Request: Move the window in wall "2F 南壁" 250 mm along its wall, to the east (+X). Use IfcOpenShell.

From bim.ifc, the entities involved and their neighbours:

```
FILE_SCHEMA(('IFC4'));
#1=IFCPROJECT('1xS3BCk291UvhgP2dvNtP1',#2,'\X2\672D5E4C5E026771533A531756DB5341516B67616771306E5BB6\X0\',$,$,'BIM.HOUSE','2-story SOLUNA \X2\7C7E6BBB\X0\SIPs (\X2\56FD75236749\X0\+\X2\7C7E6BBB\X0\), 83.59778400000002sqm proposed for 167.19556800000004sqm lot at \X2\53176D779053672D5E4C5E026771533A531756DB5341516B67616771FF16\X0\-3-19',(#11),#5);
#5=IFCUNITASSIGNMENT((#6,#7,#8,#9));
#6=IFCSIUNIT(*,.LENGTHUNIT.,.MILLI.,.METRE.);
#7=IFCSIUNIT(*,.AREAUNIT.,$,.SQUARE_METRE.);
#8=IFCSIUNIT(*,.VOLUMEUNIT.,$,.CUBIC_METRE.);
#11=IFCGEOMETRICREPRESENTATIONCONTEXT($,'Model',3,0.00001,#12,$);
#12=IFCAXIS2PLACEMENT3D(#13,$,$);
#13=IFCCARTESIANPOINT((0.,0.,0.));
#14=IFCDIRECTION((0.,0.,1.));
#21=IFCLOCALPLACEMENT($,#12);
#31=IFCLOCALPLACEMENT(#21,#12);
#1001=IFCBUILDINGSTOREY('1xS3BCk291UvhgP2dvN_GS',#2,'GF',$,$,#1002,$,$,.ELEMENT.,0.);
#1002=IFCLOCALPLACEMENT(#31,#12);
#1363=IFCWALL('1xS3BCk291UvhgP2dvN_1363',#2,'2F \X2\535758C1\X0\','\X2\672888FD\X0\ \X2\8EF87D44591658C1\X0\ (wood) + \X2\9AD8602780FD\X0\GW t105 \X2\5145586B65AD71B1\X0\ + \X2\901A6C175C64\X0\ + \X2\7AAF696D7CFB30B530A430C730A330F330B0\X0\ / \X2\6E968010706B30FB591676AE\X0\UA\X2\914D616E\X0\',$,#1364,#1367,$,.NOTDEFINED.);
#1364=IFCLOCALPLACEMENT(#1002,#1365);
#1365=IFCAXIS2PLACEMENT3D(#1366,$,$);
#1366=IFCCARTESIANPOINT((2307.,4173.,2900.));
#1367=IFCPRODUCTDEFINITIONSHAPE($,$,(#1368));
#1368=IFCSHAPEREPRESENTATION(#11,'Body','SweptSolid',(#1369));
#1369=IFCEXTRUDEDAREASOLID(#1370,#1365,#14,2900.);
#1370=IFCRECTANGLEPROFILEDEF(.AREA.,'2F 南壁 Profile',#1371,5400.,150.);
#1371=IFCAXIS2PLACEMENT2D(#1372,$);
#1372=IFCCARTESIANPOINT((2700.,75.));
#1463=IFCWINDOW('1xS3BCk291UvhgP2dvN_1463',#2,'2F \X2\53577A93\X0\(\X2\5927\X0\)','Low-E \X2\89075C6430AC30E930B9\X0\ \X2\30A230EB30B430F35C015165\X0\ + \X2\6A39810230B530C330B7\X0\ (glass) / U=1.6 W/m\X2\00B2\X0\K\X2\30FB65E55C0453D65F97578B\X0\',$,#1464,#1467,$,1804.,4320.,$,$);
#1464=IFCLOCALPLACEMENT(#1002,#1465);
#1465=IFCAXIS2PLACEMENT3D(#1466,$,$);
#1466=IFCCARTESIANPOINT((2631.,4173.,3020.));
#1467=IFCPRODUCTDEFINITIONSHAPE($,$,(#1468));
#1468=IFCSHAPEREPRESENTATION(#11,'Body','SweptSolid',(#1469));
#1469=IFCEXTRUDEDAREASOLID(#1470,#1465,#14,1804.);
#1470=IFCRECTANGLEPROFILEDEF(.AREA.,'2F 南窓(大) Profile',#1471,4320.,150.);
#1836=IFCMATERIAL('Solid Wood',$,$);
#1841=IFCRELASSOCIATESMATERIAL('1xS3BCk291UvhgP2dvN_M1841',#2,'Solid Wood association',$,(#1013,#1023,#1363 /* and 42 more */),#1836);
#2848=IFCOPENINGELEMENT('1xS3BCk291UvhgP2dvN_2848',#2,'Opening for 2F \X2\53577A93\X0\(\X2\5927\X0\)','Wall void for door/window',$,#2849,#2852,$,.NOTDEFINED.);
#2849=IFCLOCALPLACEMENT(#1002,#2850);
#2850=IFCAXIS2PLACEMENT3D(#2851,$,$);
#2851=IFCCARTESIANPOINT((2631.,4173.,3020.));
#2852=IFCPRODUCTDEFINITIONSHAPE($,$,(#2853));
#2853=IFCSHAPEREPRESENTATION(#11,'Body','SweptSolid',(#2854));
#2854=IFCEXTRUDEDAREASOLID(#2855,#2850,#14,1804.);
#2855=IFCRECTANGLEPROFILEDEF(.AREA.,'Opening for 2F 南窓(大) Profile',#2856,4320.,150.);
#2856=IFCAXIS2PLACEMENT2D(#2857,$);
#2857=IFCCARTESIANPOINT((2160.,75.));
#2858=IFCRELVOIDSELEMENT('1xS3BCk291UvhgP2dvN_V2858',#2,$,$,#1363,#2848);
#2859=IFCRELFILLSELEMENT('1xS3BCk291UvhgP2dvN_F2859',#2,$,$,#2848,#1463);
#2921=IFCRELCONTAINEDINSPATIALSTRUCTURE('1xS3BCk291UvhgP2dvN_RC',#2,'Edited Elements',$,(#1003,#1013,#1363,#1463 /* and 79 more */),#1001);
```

```python
import ifcopenshell
import ifcopenshell.api.geometry
import ifcopenshell.util.placement

model = ifcopenshell.open("bim.ifc")

window = model.by_id(1463)
opening = window.FillsVoids[0].RelatingOpeningElement
wall = opening.VoidsElements[0].RelatingBuildingElement

wall_matrix = ifcopenshell.util.placement.get_local_placement(wall.ObjectPlacement)
shift = wall_matrix[:3, 0] * 250.0
before = ifcopenshell.util.placement.get_local_placement(window.ObjectPlacement)[:3, 3].copy()

# The window is not placed relative to its opening, so move both.
for product in (opening, window):
    matrix = ifcopenshell.util.placement.get_local_placement(product.ObjectPlacement)
    matrix[:3, 3] += shift
    ifcopenshell.api.geometry.edit_object_placement(model, product=product, matrix=matrix, is_si=False)

after = ifcopenshell.util.placement.get_local_placement(window.ObjectPlacement)[:3, 3]
print("window moved by", (after - before).round(3) + 0.0)

model.write("bim_updated.ifc")
```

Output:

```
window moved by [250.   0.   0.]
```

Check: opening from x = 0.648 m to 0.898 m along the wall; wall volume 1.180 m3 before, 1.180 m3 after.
